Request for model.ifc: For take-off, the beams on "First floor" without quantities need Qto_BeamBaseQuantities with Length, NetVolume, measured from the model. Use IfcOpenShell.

First a look at what the model holds.

```python
import ifcopenshell
import ifcopenshell.util.element
import ifcopenshell.util.unit

model = ifcopenshell.open("model.ifc")
print(model.schema)
for unit_type in ("LENGTHUNIT", "AREAUNIT", "VOLUMEUNIT"):
    print(unit_type, ifcopenshell.util.unit.calculate_unit_scale(model, unit_type))
storey = next(s for s in model.by_type("IfcBuildingStorey") if s.Name == "First floor")
beams = [e for e in ifcopenshell.util.element.get_decomposition(storey) if e.is_a("IfcBeam")]
for e in sorted(beams, key=lambda e: e.id()):
    print(e.id(), e.is_a(), e.Name, list(ifcopenshell.util.element.get_psets(e, qtos_only=True)), sep=" | ")
```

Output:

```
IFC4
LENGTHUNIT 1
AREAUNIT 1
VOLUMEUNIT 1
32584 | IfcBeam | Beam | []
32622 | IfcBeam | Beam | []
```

```python
import ifcopenshell
import ifcopenshell.api.pset
import ifcopenshell.geom
import ifcopenshell.util.element
import ifcopenshell.util.shape
import ifcopenshell.util.unit

model = ifcopenshell.open("model.ifc")
unit_scale = ifcopenshell.util.unit.calculate_unit_scale(model)
volume_scale = ifcopenshell.util.unit.calculate_unit_scale(model, "VOLUMEUNIT")
settings = ifcopenshell.geom.settings()

storey = next(s for s in model.by_type("IfcBuildingStorey") if s.Name == "First floor")
beams = [e for e in ifcopenshell.util.element.get_decomposition(storey) if e.is_a("IfcBeam")]

for e in sorted(beams, key=lambda e: e.id()):
    if ifcopenshell.util.element.get_psets(e, qtos_only=True, should_inherit=False):
        continue
    # Geometry comes back in metres, in the element's own axes.
    shape = ifcopenshell.geom.create_shape(settings, e)
    values = {
        "Length": ifcopenshell.util.shape.get_max_xyz(shape.geometry) / unit_scale,
        "NetVolume": ifcopenshell.util.shape.get_volume(shape.geometry) / volume_scale,
    }
    qto = ifcopenshell.api.pset.add_qto(model, product=e, name="Qto_BeamBaseQuantities")
    ifcopenshell.api.pset.edit_qto(model, qto=qto, properties=values)
    print(e.id(), {k: round(v, 3) for k, v in values.items()})

model.write("model-out.ifc")
```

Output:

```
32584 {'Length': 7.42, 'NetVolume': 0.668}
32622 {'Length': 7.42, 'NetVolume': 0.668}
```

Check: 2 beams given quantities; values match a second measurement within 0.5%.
